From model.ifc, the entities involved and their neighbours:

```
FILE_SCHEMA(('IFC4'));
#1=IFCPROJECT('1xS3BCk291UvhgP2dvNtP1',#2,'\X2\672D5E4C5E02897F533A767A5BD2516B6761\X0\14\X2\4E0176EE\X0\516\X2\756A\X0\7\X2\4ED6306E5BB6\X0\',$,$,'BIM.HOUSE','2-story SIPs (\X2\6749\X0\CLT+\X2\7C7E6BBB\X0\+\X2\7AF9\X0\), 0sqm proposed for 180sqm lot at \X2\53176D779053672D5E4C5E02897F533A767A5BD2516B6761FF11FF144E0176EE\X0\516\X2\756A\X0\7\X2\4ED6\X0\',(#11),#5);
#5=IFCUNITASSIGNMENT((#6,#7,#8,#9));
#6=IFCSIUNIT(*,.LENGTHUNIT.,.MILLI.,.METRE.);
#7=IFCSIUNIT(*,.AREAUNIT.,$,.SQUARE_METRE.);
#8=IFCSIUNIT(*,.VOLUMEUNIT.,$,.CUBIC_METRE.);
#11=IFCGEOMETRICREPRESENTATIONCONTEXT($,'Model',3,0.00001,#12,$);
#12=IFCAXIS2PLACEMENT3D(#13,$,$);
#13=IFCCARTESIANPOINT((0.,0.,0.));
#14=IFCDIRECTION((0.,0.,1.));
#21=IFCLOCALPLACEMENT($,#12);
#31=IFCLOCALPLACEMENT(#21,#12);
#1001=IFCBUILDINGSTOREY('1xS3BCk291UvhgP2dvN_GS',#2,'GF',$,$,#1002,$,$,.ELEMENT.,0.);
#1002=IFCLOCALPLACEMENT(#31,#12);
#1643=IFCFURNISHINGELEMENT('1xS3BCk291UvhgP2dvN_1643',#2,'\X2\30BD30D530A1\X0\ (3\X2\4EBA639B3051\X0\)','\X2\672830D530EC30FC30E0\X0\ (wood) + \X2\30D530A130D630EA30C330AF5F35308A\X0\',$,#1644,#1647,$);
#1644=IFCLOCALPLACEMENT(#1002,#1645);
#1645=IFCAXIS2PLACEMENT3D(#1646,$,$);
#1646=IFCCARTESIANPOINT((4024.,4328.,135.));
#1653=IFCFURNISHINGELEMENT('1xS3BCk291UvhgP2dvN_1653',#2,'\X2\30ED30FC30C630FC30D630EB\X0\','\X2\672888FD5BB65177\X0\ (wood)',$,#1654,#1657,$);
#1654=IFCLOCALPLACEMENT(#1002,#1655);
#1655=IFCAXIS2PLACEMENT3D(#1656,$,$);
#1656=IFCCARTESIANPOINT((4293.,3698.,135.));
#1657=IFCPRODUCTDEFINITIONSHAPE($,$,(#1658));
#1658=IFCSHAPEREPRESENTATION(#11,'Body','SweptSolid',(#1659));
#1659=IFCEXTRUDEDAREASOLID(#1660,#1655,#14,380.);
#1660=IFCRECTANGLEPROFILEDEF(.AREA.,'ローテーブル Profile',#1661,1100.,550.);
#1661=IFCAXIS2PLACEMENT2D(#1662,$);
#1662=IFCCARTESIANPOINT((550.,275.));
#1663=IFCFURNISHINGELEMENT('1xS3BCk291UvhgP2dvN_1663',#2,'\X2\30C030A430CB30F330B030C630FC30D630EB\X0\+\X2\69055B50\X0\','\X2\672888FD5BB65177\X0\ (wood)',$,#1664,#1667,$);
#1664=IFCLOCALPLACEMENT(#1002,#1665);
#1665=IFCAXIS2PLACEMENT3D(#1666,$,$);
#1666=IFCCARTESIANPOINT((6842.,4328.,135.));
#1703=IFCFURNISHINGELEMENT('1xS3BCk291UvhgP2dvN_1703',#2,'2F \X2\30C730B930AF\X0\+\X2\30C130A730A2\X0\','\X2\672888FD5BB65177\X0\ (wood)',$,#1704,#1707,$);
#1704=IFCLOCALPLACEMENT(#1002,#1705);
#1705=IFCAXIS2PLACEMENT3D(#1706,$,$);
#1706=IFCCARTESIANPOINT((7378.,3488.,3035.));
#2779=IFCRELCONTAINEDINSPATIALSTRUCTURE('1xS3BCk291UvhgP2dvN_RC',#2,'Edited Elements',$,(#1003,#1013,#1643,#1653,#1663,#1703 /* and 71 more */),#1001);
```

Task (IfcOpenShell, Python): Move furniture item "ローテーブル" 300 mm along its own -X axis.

```python
import ifcopenshell
import ifcopenshell.api.geometry
import ifcopenshell.util.placement
import ifcopenshell.util.unit

model = ifcopenshell.open("model.ifc")
unit_scale = ifcopenshell.util.unit.calculate_unit_scale(model)

item = model.by_guid("1xS3BCk291UvhgP2dvN_1653")
matrix = ifcopenshell.util.placement.get_local_placement(item.ObjectPlacement)
matrix[:3, 3] -= matrix[:3, 0] * 0.3 / unit_scale
ifcopenshell.api.geometry.edit_object_placement(model, product=item, matrix=matrix, is_si=False)

print(ifcopenshell.util.placement.get_local_placement(item.ObjectPlacement).round(3) + 0.0)

model.write("model_edited.ifc")
```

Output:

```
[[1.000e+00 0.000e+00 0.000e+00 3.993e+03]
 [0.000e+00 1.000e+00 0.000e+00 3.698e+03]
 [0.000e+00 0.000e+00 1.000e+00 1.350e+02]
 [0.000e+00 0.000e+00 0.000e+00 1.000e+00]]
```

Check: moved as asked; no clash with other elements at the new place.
